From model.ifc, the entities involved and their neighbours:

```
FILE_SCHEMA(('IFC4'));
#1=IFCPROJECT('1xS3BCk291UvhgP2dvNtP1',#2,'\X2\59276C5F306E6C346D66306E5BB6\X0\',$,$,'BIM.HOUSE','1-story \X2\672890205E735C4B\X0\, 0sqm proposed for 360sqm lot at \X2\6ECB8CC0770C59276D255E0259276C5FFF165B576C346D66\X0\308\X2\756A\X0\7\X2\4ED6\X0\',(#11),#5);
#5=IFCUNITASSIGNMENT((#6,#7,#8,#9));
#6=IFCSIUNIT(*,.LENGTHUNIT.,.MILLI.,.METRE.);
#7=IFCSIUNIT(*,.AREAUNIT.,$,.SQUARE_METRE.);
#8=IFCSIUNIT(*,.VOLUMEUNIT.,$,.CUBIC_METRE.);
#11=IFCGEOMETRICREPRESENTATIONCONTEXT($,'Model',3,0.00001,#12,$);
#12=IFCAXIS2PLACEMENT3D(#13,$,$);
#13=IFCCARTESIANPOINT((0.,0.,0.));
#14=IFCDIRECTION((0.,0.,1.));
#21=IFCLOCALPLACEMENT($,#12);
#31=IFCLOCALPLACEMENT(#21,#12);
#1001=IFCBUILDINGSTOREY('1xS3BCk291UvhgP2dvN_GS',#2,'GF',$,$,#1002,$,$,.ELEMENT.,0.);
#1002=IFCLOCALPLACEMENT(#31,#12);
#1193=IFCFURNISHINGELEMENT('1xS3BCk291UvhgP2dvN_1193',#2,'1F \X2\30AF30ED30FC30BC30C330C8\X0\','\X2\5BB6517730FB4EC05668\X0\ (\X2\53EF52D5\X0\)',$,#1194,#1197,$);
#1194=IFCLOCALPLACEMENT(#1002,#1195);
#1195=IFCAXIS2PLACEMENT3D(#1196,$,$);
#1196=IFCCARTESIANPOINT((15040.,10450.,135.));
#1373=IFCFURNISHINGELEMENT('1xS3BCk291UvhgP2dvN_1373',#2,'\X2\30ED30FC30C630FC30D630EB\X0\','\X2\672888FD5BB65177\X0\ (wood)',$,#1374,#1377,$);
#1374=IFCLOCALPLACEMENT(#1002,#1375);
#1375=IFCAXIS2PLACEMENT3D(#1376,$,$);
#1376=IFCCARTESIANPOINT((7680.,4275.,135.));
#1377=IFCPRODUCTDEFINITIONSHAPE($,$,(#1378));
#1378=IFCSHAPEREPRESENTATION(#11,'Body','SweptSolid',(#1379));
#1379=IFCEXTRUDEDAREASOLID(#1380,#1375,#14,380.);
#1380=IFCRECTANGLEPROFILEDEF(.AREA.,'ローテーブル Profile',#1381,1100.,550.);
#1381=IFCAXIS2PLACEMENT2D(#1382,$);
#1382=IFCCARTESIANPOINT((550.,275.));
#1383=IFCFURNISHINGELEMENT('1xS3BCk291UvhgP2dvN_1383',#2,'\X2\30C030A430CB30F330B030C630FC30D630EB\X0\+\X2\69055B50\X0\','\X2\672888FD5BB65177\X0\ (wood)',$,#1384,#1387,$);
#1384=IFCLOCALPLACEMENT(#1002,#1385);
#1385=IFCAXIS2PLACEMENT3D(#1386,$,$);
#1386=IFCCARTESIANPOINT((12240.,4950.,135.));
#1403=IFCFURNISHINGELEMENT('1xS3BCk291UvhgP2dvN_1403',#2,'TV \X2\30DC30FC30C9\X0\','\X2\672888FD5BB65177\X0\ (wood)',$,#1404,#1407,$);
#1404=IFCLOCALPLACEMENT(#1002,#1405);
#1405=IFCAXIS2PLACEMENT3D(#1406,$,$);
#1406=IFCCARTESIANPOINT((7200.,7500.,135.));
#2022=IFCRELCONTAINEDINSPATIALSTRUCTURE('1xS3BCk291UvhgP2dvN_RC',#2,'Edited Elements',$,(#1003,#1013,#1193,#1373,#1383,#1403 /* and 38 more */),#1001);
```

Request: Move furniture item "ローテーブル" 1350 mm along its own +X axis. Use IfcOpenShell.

```python
import ifcopenshell
import ifcopenshell.api.geometry
import ifcopenshell.util.placement
import ifcopenshell.util.unit

model = ifcopenshell.open("model.ifc")
unit_scale = ifcopenshell.util.unit.calculate_unit_scale(model)

item = model.by_guid("1xS3BCk291UvhgP2dvN_1373")
matrix = ifcopenshell.util.placement.get_local_placement(item.ObjectPlacement)
matrix[:3, 3] += matrix[:3, 0] * 1.35 / unit_scale
ifcopenshell.api.geometry.edit_object_placement(model, product=item, matrix=matrix, is_si=False)

print(ifcopenshell.util.placement.get_local_placement(item.ObjectPlacement).round(3) + 0.0)

model.write("model_v2.ifc")
```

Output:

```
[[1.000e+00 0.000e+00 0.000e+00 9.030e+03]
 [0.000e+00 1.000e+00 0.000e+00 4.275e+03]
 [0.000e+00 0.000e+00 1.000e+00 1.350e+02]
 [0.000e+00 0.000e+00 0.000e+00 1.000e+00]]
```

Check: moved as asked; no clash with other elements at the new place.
